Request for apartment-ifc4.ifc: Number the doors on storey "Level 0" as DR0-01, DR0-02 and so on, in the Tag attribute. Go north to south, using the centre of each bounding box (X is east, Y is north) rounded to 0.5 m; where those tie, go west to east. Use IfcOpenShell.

First a look at what the model holds.

```python
import ifcopenshell
import ifcopenshell.util.element
import ifcopenshell.util.placement

model = ifcopenshell.open("apartment-ifc4.ifc")
print(model.schema)
storey = next(s for s in model.by_type("IfcBuildingStorey") if s.Name == "Level 0")
doors = [e for e in ifcopenshell.util.element.get_decomposition(storey) if e.is_a("IfcDoor")]
for e in sorted(doors, key=lambda e: e.id()):
    origin = ifcopenshell.util.placement.get_local_placement(e.ObjectPlacement)[:3, 3]
    print(e.id(), e.Tag, e.Name, origin.round(2) + 0.0, sep=" | ")
```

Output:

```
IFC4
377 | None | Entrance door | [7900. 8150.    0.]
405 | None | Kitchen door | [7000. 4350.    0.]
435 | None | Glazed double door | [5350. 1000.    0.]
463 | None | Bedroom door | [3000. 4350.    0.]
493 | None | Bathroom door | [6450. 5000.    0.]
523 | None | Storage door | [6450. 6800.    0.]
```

```python
import ifcopenshell
import ifcopenshell.geom
import ifcopenshell.util.element
import ifcopenshell.util.shape

model = ifcopenshell.open("apartment-ifc4.ifc")
settings = ifcopenshell.geom.settings()
settings.set("use-world-coords", True)


def centre(element):
    shape = ifcopenshell.geom.create_shape(settings, element)
    return ifcopenshell.util.shape.get_bbox_centroid(shape.geometry)


storey = next(s for s in model.by_type("IfcBuildingStorey") if s.Name == "Level 0")
doors = [e for e in ifcopenshell.util.element.get_decomposition(storey) if e.is_a("IfcDoor")]

# Insertion points can sit at a corner or the storey origin, so sort by the geometry (in metres).
centres = {e: centre(e) for e in doors}
doors.sort(key=lambda e: (-round(centres[e][1] / 0.5), centres[e][0]))

for i, e in enumerate(doors, start=1):
    number = f"DR0-{i:02d}"
    e.Tag = number
    print(e.id(), number)

model.write("apartment-ifc4_edited.ifc")
```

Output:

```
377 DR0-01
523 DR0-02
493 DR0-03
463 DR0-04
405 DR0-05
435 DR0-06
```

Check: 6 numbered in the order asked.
